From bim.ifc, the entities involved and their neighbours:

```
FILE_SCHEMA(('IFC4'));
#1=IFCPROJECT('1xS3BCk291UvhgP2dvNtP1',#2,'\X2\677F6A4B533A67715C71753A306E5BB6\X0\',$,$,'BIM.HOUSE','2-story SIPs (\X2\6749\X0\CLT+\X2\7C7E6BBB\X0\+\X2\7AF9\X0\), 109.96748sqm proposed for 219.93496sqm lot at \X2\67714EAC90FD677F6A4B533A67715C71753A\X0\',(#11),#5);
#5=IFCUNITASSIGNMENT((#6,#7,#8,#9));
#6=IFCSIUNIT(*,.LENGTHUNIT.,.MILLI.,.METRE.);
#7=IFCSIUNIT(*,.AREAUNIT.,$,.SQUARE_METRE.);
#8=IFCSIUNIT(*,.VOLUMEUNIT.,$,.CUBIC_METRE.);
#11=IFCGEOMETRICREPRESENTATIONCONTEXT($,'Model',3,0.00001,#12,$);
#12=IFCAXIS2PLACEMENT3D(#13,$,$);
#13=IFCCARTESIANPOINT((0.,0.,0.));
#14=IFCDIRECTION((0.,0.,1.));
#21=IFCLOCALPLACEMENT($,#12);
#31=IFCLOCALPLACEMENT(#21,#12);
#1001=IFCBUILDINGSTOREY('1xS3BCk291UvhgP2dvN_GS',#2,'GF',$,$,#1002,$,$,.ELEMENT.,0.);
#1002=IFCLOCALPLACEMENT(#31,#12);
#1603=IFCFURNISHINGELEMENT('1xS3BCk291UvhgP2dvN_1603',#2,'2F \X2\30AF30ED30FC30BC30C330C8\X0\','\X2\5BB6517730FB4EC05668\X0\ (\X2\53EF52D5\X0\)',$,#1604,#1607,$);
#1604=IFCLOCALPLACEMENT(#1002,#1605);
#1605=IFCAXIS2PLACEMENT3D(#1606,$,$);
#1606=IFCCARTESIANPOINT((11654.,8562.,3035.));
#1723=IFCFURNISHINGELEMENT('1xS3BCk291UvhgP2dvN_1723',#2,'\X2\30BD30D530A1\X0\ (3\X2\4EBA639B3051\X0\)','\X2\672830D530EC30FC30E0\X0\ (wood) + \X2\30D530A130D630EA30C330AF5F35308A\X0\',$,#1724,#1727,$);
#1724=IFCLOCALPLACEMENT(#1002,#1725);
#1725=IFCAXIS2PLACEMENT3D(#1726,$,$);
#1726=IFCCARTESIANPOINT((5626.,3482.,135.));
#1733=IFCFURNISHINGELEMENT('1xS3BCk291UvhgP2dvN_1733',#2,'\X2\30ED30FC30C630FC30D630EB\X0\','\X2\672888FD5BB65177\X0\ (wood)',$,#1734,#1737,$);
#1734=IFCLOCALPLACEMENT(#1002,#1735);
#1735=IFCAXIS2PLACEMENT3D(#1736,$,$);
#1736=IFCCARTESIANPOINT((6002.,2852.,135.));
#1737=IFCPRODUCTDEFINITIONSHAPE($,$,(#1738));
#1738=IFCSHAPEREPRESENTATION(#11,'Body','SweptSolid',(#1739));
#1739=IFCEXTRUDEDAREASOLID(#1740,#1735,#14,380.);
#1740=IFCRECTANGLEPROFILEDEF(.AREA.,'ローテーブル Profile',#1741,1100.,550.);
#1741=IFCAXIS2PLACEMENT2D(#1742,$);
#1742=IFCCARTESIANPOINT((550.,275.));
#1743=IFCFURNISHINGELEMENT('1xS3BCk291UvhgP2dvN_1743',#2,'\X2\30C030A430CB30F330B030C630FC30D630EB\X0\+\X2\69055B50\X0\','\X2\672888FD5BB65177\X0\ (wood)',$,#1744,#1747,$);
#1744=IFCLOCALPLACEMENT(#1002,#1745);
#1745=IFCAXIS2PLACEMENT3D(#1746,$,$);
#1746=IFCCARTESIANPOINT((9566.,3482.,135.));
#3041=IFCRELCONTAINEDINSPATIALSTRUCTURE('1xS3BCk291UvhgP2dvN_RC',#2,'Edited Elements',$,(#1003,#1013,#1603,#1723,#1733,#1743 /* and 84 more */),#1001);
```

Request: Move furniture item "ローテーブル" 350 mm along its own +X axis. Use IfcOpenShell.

```python
import ifcopenshell
import ifcopenshell.api.geometry
import ifcopenshell.util.placement
import ifcopenshell.util.unit

model = ifcopenshell.open("bim.ifc")
unit_scale = ifcopenshell.util.unit.calculate_unit_scale(model)

item = model.by_guid("1xS3BCk291UvhgP2dvN_1733")
matrix = ifcopenshell.util.placement.get_local_placement(item.ObjectPlacement)
matrix[:3, 3] += matrix[:3, 0] * 0.35 / unit_scale
ifcopenshell.api.geometry.edit_object_placement(model, product=item, matrix=matrix, is_si=False)

print(ifcopenshell.util.placement.get_local_placement(item.ObjectPlacement).round(3) + 0.0)

model.write("bim_updated.ifc")
```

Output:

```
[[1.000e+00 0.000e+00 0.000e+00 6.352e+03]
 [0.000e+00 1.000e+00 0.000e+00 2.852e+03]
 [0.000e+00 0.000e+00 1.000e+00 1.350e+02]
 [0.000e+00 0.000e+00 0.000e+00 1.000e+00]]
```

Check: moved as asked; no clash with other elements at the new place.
